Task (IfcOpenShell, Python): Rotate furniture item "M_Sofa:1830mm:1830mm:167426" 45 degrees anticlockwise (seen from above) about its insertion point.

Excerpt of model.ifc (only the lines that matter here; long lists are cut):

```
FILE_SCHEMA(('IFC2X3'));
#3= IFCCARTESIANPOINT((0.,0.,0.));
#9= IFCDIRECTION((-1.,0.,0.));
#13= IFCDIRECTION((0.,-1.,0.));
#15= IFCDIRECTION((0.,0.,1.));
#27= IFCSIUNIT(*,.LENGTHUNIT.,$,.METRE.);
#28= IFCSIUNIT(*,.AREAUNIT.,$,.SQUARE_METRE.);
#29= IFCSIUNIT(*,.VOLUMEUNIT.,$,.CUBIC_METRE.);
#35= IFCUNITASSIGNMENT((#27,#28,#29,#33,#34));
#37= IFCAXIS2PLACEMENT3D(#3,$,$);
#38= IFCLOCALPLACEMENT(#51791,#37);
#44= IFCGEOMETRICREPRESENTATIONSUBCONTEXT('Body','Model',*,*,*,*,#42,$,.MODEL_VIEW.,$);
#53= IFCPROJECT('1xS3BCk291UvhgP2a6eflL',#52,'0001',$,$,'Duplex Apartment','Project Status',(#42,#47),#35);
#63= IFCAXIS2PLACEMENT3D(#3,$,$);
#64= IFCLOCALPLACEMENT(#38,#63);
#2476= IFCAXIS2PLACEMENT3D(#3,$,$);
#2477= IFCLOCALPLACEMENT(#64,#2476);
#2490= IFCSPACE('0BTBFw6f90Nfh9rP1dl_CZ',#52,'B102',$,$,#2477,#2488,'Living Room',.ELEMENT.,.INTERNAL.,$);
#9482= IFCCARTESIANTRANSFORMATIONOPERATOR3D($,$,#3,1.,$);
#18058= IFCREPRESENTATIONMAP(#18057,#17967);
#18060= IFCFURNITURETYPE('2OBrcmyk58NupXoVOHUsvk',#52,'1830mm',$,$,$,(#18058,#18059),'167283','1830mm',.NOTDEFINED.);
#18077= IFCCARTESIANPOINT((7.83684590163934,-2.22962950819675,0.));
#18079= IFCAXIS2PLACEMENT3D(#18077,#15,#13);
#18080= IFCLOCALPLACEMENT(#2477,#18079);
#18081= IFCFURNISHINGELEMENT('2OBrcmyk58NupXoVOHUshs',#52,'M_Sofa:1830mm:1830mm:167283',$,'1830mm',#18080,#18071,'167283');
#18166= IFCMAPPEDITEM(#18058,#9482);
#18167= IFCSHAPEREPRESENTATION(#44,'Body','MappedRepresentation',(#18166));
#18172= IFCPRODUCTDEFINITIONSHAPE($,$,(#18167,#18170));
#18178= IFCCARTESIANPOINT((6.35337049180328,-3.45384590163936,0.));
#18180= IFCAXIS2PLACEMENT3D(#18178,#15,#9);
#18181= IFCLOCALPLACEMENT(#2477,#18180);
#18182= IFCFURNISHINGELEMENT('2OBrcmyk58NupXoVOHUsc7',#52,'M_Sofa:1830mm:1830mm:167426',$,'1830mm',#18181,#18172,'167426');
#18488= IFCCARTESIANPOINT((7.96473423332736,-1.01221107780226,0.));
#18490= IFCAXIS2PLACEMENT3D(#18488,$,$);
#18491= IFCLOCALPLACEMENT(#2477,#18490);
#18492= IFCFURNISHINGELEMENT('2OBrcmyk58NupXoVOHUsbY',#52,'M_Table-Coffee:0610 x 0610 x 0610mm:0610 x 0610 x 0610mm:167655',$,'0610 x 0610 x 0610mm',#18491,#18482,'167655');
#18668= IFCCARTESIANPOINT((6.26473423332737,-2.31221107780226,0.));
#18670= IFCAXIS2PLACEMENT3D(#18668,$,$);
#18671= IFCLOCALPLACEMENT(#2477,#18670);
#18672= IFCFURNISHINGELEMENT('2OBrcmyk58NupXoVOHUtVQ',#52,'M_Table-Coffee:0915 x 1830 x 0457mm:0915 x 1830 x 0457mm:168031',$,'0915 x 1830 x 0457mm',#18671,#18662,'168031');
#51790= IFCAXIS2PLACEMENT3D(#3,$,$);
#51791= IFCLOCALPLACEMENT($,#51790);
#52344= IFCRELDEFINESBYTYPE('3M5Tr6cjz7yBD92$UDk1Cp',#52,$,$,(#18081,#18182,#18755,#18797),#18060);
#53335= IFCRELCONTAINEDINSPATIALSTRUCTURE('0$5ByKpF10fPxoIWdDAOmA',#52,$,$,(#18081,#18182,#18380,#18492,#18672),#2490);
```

```python
import ifcopenshell
import ifcopenshell.api.geometry
import ifcopenshell.util.placement

model = ifcopenshell.open("model.ifc")

item = model.by_id(18182)
matrix = ifcopenshell.util.placement.get_local_placement(item.ObjectPlacement)
matrix = matrix @ ifcopenshell.util.placement.rotation(45, "Z")
ifcopenshell.api.geometry.edit_object_placement(model, product=item, matrix=matrix, is_si=False)

print(ifcopenshell.util.placement.get_local_placement(item.ObjectPlacement).round(3) + 0.0)

model.write("model-out.ifc")
```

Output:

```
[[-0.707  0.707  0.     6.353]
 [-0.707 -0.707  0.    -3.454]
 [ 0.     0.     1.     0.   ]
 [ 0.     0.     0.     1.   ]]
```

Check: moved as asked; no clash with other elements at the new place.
